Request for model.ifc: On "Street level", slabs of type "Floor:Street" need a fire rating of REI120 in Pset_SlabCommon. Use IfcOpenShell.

First a look at what the model holds.

```python
import ifcopenshell
import ifcopenshell.util.element

model = ifcopenshell.open("model.ifc")
print(model.schema)
storey = next(s for s in model.by_type("IfcBuildingStorey") if s.Name == "Street level")
slabs = [e for e in ifcopenshell.util.element.get_decomposition(storey) if e.is_a("IfcSlab")]
seen = {}
for e in slabs:
    element_type = ifcopenshell.util.element.get_type(e)
    key = (element_type.Name if element_type != e and element_type else None, ifcopenshell.util.element.get_pset(e, "Pset_SlabCommon", "FireRating"))
    seen[key] = seen.get(key, 0) + 1
for (name, value), count in sorted(seen.items(), key=str):
    print(count, "x", name, "|", value)
```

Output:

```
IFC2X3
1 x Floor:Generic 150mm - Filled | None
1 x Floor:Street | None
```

```python
import ifcopenshell
import ifcopenshell.api.pset
import ifcopenshell.util.element

model = ifcopenshell.open("model.ifc")

storey = next(s for s in model.by_type("IfcBuildingStorey") if s.Name == "Street level")
slabs = [e for e in ifcopenshell.util.element.get_decomposition(storey) if e.is_a("IfcSlab")]

count = 0
for e in slabs:
    element_type = ifcopenshell.util.element.get_type(e)
    if element_type in (None, e) or element_type.Name != "Floor:Street":
        continue
    # add_pset returns the element's existing set when there is one.
    pset = ifcopenshell.api.pset.add_pset(model, product=e, name="Pset_SlabCommon")
    ifcopenshell.api.pset.edit_pset(model, pset=pset, properties={"FireRating": "REI120"})
    count += 1

print(count, "slabs updated")

model.write("model_rev.ifc")
```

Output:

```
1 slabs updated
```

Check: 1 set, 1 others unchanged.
